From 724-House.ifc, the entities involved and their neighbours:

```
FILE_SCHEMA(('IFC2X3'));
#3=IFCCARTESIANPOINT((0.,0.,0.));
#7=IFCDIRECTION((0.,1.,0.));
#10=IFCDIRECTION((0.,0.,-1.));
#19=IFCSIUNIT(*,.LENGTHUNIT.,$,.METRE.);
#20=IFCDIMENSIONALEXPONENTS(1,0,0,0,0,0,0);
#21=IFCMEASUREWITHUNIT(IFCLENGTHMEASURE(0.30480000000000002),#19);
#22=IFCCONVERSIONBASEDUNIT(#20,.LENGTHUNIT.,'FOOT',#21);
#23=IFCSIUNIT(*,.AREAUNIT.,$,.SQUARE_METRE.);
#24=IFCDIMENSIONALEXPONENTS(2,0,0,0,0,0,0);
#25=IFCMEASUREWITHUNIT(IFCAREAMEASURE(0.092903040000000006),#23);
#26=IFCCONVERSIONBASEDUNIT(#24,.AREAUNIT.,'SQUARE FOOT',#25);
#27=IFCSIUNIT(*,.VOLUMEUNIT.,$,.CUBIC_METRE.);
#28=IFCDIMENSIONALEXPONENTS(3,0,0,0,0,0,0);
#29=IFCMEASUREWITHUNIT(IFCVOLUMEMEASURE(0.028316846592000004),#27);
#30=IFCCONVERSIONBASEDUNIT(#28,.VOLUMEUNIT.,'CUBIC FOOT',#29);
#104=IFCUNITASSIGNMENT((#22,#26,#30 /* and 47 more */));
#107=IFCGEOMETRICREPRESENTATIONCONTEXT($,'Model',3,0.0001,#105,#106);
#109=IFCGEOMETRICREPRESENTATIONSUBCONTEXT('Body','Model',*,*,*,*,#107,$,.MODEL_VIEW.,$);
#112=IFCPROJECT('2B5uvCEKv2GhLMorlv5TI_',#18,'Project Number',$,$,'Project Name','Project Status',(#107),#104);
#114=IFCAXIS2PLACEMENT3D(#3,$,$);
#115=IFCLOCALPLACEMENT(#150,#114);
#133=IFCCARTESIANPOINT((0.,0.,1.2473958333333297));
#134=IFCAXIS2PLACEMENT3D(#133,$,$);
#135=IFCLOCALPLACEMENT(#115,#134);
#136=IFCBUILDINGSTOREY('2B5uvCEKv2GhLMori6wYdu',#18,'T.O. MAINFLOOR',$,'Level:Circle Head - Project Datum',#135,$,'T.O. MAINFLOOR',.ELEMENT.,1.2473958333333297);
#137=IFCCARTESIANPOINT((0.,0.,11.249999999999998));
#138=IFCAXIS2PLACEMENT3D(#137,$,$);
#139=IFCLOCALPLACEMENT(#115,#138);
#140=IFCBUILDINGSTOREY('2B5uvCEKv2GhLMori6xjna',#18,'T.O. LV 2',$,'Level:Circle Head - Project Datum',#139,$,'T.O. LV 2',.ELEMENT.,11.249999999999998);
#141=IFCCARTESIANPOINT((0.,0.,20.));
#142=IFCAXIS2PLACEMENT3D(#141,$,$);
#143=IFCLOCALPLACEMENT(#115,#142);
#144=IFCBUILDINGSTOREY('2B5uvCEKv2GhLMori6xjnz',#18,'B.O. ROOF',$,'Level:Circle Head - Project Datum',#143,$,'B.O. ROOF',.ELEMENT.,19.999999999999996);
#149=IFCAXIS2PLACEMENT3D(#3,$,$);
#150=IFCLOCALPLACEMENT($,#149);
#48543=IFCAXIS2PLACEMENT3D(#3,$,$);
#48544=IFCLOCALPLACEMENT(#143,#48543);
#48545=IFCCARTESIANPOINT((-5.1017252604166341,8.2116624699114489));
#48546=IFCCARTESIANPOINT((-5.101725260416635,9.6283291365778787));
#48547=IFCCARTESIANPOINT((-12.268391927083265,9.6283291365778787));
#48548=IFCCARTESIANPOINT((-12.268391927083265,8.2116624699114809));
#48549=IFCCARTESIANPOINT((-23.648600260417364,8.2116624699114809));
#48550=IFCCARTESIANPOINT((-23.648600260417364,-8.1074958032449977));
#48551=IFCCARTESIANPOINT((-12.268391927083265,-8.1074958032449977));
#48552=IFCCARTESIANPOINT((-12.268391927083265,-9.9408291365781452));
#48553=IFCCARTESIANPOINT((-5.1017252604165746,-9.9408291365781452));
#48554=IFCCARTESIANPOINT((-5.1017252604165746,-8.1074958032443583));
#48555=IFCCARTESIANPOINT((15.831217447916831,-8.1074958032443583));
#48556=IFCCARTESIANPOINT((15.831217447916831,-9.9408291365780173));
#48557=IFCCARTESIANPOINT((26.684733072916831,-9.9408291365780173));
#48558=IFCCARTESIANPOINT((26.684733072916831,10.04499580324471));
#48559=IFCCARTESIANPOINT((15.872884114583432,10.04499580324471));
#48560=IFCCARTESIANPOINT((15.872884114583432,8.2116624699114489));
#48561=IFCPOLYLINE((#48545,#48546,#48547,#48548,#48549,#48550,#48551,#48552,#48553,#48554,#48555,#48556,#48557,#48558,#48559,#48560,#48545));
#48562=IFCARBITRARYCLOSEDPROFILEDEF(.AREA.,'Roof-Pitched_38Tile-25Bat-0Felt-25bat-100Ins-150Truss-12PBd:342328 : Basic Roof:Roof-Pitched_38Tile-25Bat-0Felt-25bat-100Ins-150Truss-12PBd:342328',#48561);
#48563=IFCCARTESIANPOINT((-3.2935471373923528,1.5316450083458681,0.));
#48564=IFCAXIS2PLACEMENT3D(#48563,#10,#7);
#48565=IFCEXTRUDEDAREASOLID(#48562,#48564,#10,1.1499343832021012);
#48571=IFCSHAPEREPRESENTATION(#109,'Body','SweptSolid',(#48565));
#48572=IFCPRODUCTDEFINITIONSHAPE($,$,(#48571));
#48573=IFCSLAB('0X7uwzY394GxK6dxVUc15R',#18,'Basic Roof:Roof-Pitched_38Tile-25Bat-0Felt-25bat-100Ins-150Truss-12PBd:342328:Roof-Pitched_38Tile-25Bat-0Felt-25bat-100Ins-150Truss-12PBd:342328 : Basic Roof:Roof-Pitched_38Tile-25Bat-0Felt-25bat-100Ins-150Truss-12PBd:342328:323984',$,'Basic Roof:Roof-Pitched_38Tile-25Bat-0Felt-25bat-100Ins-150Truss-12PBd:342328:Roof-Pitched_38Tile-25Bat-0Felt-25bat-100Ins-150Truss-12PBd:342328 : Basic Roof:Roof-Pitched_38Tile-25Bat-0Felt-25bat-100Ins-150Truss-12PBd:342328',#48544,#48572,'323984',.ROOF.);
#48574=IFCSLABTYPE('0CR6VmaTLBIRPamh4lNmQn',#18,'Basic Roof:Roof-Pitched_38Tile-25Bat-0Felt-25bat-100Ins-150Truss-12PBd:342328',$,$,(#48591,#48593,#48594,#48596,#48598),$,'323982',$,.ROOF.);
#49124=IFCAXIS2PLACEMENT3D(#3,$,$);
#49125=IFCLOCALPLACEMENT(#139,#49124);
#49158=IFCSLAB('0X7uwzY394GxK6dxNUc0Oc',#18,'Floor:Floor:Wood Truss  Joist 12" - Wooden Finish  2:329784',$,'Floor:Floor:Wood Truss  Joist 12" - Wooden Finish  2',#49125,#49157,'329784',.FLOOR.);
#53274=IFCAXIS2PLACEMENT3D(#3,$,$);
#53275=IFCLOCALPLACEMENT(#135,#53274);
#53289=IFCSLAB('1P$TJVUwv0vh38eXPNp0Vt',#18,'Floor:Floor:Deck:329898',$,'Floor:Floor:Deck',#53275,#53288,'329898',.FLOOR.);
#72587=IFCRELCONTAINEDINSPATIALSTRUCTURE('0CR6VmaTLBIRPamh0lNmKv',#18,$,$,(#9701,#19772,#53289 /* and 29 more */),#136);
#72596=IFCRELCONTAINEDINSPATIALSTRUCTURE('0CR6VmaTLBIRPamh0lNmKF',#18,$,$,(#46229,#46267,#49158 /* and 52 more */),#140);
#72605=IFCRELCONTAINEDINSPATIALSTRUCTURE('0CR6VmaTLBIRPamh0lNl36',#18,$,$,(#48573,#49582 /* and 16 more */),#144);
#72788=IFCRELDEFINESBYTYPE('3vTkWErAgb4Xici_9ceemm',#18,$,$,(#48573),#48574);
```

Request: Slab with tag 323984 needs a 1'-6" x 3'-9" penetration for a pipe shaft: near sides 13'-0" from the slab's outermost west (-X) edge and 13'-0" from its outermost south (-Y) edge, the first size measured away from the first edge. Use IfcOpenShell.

```python
import numpy as np
import ifcopenshell
import ifcopenshell.api.feature
import ifcopenshell.api.geometry
import ifcopenshell.api.root
import ifcopenshell.geom
import ifcopenshell.util.placement
import ifcopenshell.util.representation
import ifcopenshell.util.shape
import ifcopenshell.util.unit

model = ifcopenshell.open("724-House.ifc")
unit_scale = ifcopenshell.util.unit.calculate_unit_scale(model)
settings = ifcopenshell.geom.settings()


def volume(element):
    """Net volume in cubic metres, openings subtracted."""
    shape = ifcopenshell.geom.create_shape(settings, element)
    return ifcopenshell.util.shape.get_volume(shape.geometry)


slab = model.by_guid("0X7uwzY394GxK6dxVUc15R")
before = volume(slab)

# Extent in the slab's own axes, in metres. The edges named are its -X and -Y sides.
slab_shape = ifcopenshell.geom.create_shape(settings, slab)
vertices = ifcopenshell.util.shape.get_vertices(slab_shape.geometry)
x_min, y_min, bottom = vertices.min(axis=0)
top = vertices[:, 2].max()

opening = ifcopenshell.api.root.create_entity(model, ifc_class="IfcOpeningElement", name="Pipe shaft opening")
context = ifcopenshell.util.representation.get_context(model, "Model", "Body", "MODEL_VIEW")
width, depth = 0.4572, 1.143
outline = [(0.0, 0.0), (width, 0.0), (width, depth), (0.0, depth), (0.0, 0.0)]
# Overshoot both faces by 50 mm so the cut is clean.
shape = ifcopenshell.api.geometry.add_slab_representation(
    model, context=context, depth=top - bottom + 0.1, polyline=outline
)
ifcopenshell.api.geometry.assign_representation(model, product=opening, representation=shape)

matrix = ifcopenshell.util.placement.get_local_placement(slab.ObjectPlacement)
matrix[:, 3] = matrix @ np.append(np.array([x_min + 3.9624, y_min + 3.9624, bottom - 0.05]) / unit_scale, 1.0)
ifcopenshell.api.geometry.edit_object_placement(model, product=opening, matrix=matrix, is_si=False)
ifcopenshell.api.feature.add_feature(model, feature=opening, element=slab)

after = volume(slab)

print(f"slab volume {before:.3f} -> {after:.3f} m3")

model.write("724-House_rev.ifc")
```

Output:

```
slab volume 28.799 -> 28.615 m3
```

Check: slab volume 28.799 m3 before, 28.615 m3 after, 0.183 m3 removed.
